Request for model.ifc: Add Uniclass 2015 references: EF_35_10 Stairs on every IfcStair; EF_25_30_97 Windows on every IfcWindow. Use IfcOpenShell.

First a look at what the model holds.

```python
import ifcopenshell

model = ifcopenshell.open("model.ifc")
print(model.schema)
print("classifications:", [c.Name for c in model.by_type("IfcClassification")])
for ifc_class in ("IfcDoor", "IfcRoof", "IfcStair", "IfcWall", "IfcWindow"):
    print(ifc_class, len(model.by_type(ifc_class)))
```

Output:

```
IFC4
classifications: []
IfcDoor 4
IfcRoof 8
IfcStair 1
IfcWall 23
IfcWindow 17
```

```python
import ifcopenshell
import ifcopenshell.api.classification

model = ifcopenshell.open("model.ifc")

system = ifcopenshell.api.classification.add_classification(model, classification="Uniclass 2015")

codes = {
    "IfcStair": ("EF_35_10", "Stairs"),
    "IfcWindow": ("EF_25_30_97", "Windows"),
}
for ifc_class, (code, name) in codes.items():
    products = model.by_type(ifc_class)
    ifcopenshell.api.classification.add_reference(
        model, products=products, classification=system, identification=code, name=name
    )
    print(code, len(products))

model.write("model_updated.ifc")
```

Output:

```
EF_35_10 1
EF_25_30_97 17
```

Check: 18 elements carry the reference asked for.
